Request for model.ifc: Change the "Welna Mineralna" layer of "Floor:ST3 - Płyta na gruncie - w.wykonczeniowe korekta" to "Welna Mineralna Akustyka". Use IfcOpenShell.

First a look at what the model holds.

```python
import ifcopenshell
import ifcopenshell.util.element

model = ifcopenshell.open("model.ifc")
print(model.schema)
for layer_set in model.by_type("IfcMaterialLayerSet"):
    if layer_set.LayerSetName == "Floor:ST3 - Płyta na gruncie - w.wykonczeniowe korekta":
        for layer in layer_set.MaterialLayers:
            print(layer.id(), layer.Material and layer.Material.Name, layer.LayerThickness, sep=" | ")
        print(len(ifcopenshell.util.element.get_elements_by_material(model, layer_set)), "elements and types use it")
print(sorted(m.Name for m in model.by_type("IfcMaterial") if m.Name)[:60])
```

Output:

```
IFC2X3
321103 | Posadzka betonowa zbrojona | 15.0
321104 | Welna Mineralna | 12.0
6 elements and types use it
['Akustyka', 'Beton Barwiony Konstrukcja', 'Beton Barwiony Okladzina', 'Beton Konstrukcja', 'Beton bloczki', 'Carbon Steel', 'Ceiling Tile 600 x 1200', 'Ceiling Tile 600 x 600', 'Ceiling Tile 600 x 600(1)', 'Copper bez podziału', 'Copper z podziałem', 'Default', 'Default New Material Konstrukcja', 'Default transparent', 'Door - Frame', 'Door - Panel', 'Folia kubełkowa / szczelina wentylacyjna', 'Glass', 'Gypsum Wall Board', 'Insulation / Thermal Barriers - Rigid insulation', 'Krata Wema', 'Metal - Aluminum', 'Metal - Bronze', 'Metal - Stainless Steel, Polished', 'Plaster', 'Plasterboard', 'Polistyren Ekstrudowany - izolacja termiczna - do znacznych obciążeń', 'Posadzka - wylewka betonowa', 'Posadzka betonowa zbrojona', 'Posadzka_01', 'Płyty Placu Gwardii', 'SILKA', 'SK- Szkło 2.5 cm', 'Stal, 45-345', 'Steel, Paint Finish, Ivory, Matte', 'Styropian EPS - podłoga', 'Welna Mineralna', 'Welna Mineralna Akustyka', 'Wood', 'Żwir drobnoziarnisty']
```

```python
import ifcopenshell
import ifcopenshell.api.material

model = ifcopenshell.open("model.ifc")

layer_set = next(s for s in model.by_type("IfcMaterialLayerSet") if s.LayerSetName == "Floor:ST3 - Płyta na gruncie - w.wykonczeniowe korekta")
layer = next(l for l in layer_set.MaterialLayers if l.Material and l.Material.Name == "Welna Mineralna")
material = next(m for m in model.by_type("IfcMaterial") if m.Name == "Welna Mineralna Akustyka")

# Point this one layer at the other material; renaming the old one would change it everywhere.
ifcopenshell.api.material.edit_layer(model, layer=layer, attributes={}, material=material)

print([l.Material.Name if l.Material else None for l in layer_set.MaterialLayers])

model.write("model-out.ifc")
```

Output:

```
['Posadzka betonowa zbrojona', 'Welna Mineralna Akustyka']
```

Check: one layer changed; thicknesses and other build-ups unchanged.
